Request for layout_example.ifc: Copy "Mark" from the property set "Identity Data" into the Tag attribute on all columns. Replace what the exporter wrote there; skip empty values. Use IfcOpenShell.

First a look at what the model holds.

```python
import ifcopenshell
import ifcopenshell.util.element

model = ifcopenshell.open("layout_example.ifc")
print(model.schema)
columns = model.by_type("IfcColumn")
print(len(columns), "columns")
for e in columns[:8]:
    source = ifcopenshell.util.element.get_pset(e, "Identity Data", "Mark")
    target = e.Tag
    print(e.id(), repr(source), repr(target), sep=" | ")
```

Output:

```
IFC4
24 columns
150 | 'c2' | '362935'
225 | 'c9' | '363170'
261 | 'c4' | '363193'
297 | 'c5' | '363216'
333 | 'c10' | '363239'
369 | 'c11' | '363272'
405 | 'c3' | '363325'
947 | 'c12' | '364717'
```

```python
import ifcopenshell
import ifcopenshell.util.element

model = ifcopenshell.open("layout_example.ifc")

count = 0
for e in model.by_type("IfcColumn"):
    value = ifcopenshell.util.element.get_pset(e, "Identity Data", "Mark")
    current = e.Tag
    if not value or not value.strip() or current == value:
        continue
    e.Tag = value
    count += 1

print(count, "columns updated")

model.write("layout_example_updated.ifc")
```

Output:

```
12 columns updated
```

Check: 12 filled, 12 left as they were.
